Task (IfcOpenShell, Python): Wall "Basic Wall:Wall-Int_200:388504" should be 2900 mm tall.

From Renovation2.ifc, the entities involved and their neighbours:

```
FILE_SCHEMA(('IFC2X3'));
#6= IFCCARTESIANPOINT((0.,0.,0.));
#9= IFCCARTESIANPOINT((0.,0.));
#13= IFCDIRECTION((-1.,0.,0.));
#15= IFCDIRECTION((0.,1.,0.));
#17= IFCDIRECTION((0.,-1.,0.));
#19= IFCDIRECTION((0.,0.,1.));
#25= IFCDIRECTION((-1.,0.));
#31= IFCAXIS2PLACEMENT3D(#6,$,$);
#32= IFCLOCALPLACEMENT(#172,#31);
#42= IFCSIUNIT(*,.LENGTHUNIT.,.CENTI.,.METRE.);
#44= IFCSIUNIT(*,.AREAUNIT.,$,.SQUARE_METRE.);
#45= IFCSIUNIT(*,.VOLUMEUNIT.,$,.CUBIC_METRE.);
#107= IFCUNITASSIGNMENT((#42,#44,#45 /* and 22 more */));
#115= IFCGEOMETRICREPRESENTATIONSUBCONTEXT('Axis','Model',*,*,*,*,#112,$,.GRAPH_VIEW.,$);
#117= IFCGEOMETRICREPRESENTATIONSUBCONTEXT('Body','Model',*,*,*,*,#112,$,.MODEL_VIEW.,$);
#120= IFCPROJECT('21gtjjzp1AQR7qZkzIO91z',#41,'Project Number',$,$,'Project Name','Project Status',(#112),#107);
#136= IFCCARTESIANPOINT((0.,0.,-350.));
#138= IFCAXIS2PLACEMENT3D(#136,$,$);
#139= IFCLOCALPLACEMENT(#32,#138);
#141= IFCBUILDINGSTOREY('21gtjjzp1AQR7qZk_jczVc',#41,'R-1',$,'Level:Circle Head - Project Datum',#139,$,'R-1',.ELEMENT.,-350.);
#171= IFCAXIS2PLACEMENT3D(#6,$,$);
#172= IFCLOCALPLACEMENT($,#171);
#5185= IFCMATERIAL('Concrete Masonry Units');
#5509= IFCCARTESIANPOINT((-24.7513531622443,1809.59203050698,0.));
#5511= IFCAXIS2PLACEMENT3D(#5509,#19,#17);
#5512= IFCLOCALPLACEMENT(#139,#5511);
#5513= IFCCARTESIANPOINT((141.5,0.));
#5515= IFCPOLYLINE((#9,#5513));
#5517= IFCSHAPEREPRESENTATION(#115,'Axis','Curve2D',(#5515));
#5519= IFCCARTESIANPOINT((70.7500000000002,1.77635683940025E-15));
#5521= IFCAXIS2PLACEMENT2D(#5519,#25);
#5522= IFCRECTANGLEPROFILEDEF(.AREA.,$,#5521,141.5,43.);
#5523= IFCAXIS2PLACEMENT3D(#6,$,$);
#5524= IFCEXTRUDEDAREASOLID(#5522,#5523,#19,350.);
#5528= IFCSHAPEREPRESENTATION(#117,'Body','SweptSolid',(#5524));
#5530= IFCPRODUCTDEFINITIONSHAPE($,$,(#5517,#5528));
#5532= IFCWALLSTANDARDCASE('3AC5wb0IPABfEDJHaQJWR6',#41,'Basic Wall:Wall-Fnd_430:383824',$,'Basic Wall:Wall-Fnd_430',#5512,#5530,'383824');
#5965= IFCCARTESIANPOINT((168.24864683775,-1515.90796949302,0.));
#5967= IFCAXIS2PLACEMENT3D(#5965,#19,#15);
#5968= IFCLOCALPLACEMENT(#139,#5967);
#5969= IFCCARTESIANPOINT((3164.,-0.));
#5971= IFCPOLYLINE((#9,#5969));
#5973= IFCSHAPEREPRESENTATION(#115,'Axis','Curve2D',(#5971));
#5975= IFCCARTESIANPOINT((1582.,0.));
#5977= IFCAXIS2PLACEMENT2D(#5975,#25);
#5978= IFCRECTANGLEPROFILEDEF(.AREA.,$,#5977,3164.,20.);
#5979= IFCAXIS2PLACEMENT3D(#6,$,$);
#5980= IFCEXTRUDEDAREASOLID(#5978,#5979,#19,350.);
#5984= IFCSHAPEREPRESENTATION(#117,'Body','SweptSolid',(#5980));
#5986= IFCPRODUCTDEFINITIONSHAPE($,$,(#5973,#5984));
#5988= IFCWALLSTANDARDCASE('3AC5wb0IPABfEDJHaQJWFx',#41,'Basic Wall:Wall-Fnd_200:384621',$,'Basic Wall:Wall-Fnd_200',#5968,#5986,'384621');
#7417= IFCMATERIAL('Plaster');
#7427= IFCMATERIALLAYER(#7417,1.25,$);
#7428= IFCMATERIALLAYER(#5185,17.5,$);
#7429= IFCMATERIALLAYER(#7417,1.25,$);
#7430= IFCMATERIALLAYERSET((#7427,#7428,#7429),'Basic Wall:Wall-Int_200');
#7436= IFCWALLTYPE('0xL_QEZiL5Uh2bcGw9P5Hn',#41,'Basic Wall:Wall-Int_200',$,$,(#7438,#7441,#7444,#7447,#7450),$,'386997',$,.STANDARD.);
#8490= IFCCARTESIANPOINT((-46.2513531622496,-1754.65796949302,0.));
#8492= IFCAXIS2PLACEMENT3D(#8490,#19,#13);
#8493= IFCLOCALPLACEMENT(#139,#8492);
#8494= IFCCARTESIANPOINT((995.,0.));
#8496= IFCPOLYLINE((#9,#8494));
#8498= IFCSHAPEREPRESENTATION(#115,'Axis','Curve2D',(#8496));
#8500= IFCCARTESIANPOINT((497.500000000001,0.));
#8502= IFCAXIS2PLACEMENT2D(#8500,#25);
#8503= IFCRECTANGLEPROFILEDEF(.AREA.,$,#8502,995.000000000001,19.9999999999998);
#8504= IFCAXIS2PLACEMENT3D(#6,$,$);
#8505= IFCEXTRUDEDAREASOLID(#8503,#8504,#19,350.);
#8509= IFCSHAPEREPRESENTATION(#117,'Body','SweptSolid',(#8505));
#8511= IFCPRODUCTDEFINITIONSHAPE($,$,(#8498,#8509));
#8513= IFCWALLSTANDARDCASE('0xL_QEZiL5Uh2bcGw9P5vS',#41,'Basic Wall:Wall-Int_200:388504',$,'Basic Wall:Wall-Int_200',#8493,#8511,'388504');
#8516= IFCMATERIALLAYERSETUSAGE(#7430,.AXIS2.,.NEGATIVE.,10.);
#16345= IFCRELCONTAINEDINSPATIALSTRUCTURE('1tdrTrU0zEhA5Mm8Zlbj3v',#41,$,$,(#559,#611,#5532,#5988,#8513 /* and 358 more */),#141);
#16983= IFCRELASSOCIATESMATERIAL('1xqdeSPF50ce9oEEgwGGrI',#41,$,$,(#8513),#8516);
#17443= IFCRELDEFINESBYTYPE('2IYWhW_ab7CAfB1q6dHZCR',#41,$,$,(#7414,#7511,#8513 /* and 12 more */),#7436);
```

```python
import ifcopenshell
import ifcopenshell.geom
import ifcopenshell.util.representation
import ifcopenshell.util.shape
import ifcopenshell.util.unit

model = ifcopenshell.open("Renovation2.ifc")
unit_scale = ifcopenshell.util.unit.calculate_unit_scale(model)
settings = ifcopenshell.geom.settings()


def volume(element):
    """Net volume in cubic metres, openings subtracted."""
    shape = ifcopenshell.geom.create_shape(settings, element)
    return ifcopenshell.util.shape.get_volume(shape.geometry)


wall = model.by_id(8513)
before = volume(wall)

body = ifcopenshell.util.representation.get_representation(wall, "Model", "Body")
solid = body.Items[0]
old_height = solid.Depth
solid.Depth = 2.9 / unit_scale
after = volume(wall)

print(f"height {old_height:g} -> {solid.Depth:g}, volume {before:.3f} -> {after:.3f} m3")

model.write("Renovation2_rev.ifc")
```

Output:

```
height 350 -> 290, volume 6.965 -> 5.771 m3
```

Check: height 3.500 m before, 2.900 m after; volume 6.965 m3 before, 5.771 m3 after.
